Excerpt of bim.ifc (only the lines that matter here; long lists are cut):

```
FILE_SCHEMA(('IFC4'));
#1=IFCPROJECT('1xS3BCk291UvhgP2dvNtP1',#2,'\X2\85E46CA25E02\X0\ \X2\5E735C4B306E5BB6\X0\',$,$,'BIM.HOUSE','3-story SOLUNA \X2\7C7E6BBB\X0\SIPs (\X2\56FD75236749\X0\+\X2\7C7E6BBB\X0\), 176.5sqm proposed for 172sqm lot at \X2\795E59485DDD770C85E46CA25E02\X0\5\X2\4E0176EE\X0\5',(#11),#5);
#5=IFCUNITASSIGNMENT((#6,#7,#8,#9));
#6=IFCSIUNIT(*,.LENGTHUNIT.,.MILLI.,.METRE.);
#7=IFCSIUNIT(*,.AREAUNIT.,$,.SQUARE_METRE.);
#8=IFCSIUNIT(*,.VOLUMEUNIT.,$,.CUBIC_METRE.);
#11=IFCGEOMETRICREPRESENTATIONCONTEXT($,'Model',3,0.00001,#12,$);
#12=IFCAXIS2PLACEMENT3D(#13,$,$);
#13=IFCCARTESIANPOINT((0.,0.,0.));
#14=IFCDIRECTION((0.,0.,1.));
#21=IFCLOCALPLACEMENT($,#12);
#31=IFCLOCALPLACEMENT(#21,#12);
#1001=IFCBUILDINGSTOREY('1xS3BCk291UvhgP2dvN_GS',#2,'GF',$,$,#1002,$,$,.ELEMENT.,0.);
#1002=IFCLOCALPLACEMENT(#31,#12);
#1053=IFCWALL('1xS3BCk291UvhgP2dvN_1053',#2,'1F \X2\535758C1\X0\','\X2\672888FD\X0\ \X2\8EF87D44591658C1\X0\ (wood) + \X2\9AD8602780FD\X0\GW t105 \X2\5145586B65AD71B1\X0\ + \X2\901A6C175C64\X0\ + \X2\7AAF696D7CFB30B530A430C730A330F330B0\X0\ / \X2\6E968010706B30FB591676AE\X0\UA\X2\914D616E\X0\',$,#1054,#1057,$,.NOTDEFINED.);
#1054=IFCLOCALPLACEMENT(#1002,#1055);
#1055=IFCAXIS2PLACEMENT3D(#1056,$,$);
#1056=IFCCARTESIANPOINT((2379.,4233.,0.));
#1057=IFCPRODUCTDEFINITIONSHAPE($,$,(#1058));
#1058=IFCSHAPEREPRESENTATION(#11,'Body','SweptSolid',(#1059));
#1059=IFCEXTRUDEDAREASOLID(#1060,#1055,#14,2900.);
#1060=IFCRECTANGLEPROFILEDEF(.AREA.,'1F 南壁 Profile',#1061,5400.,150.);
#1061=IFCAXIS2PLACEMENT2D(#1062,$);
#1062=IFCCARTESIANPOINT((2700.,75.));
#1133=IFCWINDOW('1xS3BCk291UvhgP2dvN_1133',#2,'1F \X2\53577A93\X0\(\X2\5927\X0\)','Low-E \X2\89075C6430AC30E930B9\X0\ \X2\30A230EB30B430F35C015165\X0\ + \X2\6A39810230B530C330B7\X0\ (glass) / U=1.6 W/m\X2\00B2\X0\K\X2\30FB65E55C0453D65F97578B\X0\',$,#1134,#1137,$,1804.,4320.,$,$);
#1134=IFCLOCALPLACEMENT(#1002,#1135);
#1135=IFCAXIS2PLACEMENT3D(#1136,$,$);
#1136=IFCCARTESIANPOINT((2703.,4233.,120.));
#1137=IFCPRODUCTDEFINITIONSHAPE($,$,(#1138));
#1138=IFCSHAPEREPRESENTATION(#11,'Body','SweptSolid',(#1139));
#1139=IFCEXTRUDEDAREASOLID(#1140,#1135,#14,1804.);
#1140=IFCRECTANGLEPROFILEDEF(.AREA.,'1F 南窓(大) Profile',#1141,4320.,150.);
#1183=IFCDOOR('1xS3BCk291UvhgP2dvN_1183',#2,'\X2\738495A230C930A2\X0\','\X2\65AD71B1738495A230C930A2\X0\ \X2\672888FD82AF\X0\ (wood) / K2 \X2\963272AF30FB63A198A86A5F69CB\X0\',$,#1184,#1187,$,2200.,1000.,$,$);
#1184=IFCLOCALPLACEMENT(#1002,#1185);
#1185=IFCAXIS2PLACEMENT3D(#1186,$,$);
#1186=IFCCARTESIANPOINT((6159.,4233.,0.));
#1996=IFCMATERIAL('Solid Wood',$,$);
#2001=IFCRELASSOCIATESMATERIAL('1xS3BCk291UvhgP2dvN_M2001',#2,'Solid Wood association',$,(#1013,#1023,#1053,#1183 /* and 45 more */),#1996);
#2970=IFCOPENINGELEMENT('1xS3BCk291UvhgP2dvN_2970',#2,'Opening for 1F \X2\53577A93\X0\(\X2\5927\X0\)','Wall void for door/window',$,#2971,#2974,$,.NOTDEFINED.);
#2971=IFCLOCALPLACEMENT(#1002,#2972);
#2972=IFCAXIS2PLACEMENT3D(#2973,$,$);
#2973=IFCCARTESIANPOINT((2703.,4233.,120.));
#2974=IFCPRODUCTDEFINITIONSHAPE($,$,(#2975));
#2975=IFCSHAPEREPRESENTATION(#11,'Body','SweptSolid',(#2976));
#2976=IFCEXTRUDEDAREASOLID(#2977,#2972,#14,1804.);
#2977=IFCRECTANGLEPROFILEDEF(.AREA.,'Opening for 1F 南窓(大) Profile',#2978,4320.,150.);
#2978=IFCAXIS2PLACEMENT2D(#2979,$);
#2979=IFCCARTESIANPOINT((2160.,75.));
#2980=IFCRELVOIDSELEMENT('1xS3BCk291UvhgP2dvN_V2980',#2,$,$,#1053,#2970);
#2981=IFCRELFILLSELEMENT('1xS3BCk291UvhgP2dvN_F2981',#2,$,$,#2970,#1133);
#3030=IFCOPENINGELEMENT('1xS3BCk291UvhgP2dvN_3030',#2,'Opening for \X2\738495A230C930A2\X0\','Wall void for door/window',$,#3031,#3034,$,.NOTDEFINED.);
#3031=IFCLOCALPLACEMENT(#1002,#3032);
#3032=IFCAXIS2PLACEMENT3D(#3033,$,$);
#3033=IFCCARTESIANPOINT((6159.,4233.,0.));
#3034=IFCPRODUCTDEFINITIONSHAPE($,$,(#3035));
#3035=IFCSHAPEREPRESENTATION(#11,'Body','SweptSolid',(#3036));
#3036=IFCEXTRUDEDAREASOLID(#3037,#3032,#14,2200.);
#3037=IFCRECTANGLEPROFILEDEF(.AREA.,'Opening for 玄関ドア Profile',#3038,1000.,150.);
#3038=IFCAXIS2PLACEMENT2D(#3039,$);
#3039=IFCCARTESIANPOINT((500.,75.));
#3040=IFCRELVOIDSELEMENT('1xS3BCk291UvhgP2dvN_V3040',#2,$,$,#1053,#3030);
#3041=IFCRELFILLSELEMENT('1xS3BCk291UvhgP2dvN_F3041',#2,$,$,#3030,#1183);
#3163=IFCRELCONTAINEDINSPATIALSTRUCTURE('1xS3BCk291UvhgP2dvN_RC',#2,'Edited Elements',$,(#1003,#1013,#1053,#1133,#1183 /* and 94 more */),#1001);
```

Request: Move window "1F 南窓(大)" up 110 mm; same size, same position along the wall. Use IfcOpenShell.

```python
import numpy as np
import ifcopenshell
import ifcopenshell.api.geometry
import ifcopenshell.util.placement
import ifcopenshell.util.unit

model = ifcopenshell.open("bim.ifc")
unit_scale = ifcopenshell.util.unit.calculate_unit_scale(model)

window = model.by_id(1133)
opening = window.FillsVoids[0].RelatingOpeningElement
dz = 0.11 / unit_scale

shift = np.array([0.0, 0.0, dz])
# The window is not placed relative to its opening, so move both.
for product in (opening, window):
    matrix = ifcopenshell.util.placement.get_local_placement(product.ObjectPlacement)
    matrix[:3, 3] += shift
    ifcopenshell.api.geometry.edit_object_placement(model, product=product, matrix=matrix, is_si=False)

print(f"moved by {dz * unit_scale:+.3f} m")

model.write("bim_updated.ifc")
```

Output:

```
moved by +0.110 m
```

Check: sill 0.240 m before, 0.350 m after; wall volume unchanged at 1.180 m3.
